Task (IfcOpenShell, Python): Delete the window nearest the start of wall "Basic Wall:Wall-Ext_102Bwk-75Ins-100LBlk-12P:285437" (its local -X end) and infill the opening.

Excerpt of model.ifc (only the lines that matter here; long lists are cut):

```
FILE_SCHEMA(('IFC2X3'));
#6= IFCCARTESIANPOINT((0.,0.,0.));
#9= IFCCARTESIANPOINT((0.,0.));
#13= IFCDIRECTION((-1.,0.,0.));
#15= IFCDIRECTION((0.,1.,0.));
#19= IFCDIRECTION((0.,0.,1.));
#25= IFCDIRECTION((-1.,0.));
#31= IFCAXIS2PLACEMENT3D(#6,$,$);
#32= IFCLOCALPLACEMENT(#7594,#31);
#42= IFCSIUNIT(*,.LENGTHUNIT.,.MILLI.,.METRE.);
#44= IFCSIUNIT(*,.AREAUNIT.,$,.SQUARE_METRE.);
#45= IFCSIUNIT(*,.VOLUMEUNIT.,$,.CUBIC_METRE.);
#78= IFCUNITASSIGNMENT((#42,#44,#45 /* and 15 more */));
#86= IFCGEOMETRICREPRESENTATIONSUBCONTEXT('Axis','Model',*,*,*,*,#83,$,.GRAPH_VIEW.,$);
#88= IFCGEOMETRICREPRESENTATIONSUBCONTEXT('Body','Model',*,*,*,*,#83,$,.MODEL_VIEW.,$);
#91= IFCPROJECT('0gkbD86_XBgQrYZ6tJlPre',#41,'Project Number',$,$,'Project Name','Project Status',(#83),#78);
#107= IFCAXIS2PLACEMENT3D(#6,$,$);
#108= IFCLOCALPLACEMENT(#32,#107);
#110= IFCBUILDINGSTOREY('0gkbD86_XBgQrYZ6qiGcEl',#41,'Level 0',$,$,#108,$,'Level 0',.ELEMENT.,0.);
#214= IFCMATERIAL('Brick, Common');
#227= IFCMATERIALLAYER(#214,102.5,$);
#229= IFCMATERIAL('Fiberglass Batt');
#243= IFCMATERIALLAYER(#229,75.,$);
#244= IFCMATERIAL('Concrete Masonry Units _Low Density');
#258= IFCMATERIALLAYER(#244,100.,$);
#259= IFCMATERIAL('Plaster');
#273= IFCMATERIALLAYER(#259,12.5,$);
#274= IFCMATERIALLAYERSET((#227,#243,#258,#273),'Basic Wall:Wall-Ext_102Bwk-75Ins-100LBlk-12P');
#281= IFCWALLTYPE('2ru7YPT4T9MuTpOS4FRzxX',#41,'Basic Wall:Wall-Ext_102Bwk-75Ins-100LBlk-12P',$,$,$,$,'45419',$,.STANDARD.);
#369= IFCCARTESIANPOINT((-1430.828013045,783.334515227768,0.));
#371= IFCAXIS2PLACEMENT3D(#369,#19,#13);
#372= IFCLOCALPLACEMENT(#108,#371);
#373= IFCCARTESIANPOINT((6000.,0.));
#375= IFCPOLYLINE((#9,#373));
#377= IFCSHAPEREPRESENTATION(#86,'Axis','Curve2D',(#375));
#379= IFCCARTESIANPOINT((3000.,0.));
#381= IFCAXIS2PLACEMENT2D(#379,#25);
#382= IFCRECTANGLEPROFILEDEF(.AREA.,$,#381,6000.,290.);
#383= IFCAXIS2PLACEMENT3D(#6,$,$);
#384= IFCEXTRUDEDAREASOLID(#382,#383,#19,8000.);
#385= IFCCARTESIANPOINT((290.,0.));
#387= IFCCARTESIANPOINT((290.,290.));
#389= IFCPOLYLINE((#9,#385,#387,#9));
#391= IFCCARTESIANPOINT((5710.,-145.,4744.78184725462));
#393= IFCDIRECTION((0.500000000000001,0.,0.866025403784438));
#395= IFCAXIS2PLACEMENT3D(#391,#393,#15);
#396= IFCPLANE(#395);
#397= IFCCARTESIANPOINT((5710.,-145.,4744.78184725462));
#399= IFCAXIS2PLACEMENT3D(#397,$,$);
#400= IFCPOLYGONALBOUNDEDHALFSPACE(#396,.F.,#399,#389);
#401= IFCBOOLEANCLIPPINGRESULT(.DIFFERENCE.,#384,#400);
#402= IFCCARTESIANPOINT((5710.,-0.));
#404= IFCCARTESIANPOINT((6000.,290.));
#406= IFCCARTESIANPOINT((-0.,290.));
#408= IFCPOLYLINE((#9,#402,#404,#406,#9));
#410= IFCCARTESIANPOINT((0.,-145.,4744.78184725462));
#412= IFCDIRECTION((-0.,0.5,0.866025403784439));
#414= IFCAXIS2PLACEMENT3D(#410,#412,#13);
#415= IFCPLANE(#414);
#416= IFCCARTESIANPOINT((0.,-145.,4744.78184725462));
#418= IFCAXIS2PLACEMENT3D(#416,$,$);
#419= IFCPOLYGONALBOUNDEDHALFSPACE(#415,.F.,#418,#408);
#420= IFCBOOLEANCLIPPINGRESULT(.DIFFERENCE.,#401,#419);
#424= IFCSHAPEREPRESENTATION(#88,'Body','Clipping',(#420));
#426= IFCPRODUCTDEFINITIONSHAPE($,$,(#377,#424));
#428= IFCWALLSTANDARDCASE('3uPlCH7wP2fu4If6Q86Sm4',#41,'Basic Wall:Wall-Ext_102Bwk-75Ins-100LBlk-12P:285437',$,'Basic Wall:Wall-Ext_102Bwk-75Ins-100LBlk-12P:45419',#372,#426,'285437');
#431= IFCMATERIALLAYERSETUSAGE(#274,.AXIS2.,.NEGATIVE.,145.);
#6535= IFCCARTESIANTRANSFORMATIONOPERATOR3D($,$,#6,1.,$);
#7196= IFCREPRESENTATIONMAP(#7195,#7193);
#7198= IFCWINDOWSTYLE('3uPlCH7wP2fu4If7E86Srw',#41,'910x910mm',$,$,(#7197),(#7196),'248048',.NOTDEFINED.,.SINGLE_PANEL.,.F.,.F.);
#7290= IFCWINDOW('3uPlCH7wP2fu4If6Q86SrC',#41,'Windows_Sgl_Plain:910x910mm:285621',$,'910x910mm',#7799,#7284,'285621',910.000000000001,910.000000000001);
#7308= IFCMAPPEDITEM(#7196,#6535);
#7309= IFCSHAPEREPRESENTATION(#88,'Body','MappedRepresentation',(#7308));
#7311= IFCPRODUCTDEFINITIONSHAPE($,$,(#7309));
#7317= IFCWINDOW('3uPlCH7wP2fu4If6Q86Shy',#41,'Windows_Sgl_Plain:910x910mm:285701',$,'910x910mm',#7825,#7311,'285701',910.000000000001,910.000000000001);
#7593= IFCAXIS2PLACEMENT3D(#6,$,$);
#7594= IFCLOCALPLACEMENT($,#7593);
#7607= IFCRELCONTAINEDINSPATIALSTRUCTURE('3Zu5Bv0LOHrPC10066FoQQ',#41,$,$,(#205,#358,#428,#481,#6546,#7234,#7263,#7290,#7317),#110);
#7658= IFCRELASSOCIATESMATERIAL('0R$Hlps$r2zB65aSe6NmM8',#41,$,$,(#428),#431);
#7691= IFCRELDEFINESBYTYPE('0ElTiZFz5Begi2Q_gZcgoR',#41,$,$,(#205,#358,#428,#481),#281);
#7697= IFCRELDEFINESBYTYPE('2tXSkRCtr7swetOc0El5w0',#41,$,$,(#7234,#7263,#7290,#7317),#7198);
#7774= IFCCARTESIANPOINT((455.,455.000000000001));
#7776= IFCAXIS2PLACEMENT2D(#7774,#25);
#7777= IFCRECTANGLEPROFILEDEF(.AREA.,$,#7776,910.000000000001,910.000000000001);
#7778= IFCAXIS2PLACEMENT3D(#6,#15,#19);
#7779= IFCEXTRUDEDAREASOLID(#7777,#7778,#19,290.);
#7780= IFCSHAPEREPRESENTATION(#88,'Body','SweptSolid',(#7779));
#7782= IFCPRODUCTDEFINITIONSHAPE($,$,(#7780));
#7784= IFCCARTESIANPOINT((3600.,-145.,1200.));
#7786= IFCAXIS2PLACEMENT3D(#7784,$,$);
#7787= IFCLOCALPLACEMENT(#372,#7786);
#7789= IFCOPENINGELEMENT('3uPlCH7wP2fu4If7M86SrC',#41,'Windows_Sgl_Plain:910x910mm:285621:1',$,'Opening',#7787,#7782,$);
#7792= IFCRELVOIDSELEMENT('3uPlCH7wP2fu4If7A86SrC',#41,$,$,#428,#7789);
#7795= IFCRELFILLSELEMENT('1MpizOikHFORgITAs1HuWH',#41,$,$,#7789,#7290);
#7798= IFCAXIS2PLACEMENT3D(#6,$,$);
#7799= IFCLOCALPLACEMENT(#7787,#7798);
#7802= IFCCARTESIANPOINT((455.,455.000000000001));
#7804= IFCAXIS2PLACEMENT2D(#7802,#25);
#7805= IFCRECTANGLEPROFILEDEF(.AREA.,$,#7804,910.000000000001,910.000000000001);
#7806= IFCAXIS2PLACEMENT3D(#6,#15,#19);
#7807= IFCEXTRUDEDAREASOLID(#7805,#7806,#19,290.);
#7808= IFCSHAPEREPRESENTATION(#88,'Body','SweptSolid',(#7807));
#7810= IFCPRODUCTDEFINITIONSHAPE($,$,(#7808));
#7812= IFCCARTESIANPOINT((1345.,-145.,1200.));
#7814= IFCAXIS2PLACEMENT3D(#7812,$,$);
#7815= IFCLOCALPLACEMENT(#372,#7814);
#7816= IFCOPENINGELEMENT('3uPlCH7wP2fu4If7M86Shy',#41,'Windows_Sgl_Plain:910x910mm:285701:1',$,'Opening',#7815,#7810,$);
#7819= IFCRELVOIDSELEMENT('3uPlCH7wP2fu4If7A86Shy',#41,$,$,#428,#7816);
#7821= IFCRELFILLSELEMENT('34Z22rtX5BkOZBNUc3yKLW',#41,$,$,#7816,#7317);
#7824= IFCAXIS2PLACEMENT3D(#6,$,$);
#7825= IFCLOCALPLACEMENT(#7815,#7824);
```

```python
import ifcopenshell
import ifcopenshell.api.feature
import ifcopenshell.api.root
import ifcopenshell.geom
import ifcopenshell.util.shape

model = ifcopenshell.open("model.ifc")
settings = ifcopenshell.geom.settings()


def volume(element):
    """Net volume in cubic metres, openings subtracted."""
    shape = ifcopenshell.geom.create_shape(settings, element)
    return ifcopenshell.util.shape.get_volume(shape.geometry)


window = model.by_guid("3uPlCH7wP2fu4If6Q86Shy")
opening = window.FillsVoids[0].RelatingOpeningElement
wall = opening.VoidsElements[0].RelatingBuildingElement
before = volume(wall)

ifcopenshell.api.root.remove_product(model, product=window)
ifcopenshell.api.feature.remove_feature(model, feature=opening)

after = volume(wall)

print(f"wall volume {before:.3f} -> {after:.3f} m3")

model.write("model_rev.ifc")
```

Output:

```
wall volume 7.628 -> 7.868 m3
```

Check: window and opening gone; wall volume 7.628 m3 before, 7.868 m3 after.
